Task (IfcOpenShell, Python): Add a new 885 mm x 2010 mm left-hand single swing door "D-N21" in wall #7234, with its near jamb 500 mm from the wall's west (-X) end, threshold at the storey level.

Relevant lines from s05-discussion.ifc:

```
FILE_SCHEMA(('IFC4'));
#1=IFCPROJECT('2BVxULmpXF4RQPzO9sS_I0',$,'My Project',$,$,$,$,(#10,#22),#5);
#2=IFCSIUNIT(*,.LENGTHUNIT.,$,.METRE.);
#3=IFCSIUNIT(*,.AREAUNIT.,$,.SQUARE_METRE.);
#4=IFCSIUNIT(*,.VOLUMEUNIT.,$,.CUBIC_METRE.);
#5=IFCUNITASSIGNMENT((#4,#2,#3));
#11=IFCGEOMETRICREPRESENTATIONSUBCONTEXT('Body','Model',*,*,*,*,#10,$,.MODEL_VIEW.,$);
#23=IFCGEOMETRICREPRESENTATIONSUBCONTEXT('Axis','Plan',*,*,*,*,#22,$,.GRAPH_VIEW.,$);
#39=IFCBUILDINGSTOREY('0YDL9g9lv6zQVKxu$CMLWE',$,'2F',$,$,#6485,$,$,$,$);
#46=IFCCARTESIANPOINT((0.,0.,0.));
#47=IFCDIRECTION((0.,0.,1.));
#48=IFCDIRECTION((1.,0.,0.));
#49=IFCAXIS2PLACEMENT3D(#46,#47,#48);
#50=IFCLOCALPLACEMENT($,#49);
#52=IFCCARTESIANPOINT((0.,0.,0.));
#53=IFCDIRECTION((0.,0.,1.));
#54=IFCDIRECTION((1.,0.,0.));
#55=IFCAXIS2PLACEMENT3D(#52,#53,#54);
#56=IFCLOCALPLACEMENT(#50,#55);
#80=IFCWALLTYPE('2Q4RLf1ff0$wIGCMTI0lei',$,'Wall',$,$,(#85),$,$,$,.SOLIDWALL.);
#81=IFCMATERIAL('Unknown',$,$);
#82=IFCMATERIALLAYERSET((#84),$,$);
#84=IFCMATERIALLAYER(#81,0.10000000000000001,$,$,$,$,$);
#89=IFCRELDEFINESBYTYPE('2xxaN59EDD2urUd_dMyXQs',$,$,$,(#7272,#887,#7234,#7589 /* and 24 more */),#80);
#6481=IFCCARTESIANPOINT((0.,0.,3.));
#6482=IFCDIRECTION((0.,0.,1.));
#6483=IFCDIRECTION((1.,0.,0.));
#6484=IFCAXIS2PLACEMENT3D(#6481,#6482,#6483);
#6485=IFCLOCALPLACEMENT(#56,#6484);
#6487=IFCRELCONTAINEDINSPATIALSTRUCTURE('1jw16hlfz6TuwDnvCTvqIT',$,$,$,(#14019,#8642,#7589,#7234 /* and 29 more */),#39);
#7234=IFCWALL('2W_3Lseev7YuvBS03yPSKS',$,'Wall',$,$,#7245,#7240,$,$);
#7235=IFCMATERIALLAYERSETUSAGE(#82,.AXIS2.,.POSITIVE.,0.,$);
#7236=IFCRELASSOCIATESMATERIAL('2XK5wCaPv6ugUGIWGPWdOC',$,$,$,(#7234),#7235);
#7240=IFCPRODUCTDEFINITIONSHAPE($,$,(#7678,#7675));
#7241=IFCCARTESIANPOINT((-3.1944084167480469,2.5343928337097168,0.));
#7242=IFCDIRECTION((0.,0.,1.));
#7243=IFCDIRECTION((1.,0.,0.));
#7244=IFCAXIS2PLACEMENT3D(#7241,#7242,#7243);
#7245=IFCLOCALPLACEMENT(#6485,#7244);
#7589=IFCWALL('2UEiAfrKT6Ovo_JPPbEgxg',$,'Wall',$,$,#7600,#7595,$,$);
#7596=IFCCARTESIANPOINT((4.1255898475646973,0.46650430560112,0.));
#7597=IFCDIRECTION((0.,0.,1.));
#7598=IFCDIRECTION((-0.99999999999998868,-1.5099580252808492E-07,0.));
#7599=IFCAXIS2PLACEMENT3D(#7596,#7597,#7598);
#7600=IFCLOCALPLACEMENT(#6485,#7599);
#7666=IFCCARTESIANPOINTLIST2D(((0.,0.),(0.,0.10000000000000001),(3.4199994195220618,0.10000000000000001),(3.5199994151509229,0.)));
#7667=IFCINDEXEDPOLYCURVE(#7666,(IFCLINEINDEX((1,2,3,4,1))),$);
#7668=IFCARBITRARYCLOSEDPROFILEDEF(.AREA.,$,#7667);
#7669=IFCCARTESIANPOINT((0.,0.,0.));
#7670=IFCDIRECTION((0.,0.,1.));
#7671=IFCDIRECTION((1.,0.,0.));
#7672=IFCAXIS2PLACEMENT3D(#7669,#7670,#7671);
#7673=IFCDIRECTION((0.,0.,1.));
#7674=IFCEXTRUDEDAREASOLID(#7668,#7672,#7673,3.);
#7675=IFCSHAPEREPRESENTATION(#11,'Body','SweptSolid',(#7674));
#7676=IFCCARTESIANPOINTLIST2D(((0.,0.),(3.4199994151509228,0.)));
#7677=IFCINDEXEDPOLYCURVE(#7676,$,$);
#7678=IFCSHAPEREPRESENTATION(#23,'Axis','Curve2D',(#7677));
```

```python
import numpy as np
import ifcopenshell
import ifcopenshell.api.feature
import ifcopenshell.api.geometry
import ifcopenshell.api.root
import ifcopenshell.api.spatial
import ifcopenshell.geom
import ifcopenshell.util.element
import ifcopenshell.util.placement
import ifcopenshell.util.representation
import ifcopenshell.util.shape
import ifcopenshell.util.unit

model = ifcopenshell.open("s05-discussion.ifc")
unit_scale = ifcopenshell.util.unit.calculate_unit_scale(model)
settings = ifcopenshell.geom.settings()


def volume(element):
    """Net volume in cubic metres, openings subtracted."""
    shape = ifcopenshell.geom.create_shape(settings, element)
    return ifcopenshell.util.shape.get_volume(shape.geometry)


wall = model.by_guid("2W_3Lseev7YuvBS03yPSKS")
storey = ifcopenshell.util.element.get_container(wall, ifc_class="IfcBuildingStorey")
context = ifcopenshell.util.representation.get_context(model, "Model", "Body", "MODEL_VIEW")
before = volume(wall)

width, height, from_end, sill = 0.885, 2.01, 0.5, 0.0  # metres

# The wall runs along its own X axis, and the end named is its -X end.
wall_shape = ifcopenshell.geom.create_shape(settings, wall)
x, y, z = ifcopenshell.util.shape.get_vertices(wall_shape.geometry).T
start = x.min() + from_end
face, thickness = float(y.min()), float(y.max() - y.min())
wall_matrix = ifcopenshell.util.placement.get_local_placement(wall.ObjectPlacement)
level = ifcopenshell.util.placement.get_local_placement(storey.ObjectPlacement)[2, 3]


def in_wall(x, y):
    """Placement at x, y metres in the wall's axes, at sill height."""
    matrix = wall_matrix.copy()
    matrix[:, 3] = wall_matrix @ np.array([x / unit_scale, y / unit_scale, 0.0, 1.0])
    matrix[2, 3] = level + sill / unit_scale
    return matrix


# Opening: a box that overshoots both wall faces by 50 mm.
opening = ifcopenshell.api.root.create_entity(model, ifc_class="IfcOpeningElement", predefined_type="OPENING")
box = ifcopenshell.api.geometry.add_wall_representation(
    model, context=context, length=width, height=height, thickness=thickness + 0.1
)
ifcopenshell.api.geometry.assign_representation(model, product=opening, representation=box)
ifcopenshell.api.geometry.edit_object_placement(model, product=opening, matrix=in_wall(start, face - 0.05), is_si=False)
ifcopenshell.api.feature.add_feature(model, feature=opening, element=wall)

door = ifcopenshell.api.root.create_entity(model, ifc_class="IfcDoor", name="D-N21", predefined_type="DOOR")
door.OverallWidth, door.OverallHeight = width / unit_scale, height / unit_scale
door.OperationType = "SINGLE_SWING_LEFT"
body = ifcopenshell.api.geometry.add_door_representation(
    model,
    context=context,
    overall_width=door.OverallWidth,
    overall_height=door.OverallHeight,
    operation_type="SINGLE_SWING_LEFT",
    lining_properties={"LiningDepth": thickness / unit_scale, "ThresholdDepth": thickness / unit_scale},
)
ifcopenshell.api.geometry.assign_representation(model, product=door, representation=body)
ifcopenshell.api.spatial.assign_container(model, products=[door], relating_structure=storey)
ifcopenshell.api.feature.add_filling(model, opening=opening, element=door)

# The lining spans the wall, so the door starts at the wall face.
ifcopenshell.api.geometry.edit_object_placement(model, product=door, matrix=in_wall(start, face), is_si=False)

after = volume(wall)

print(f"wall volume {before:.3f} -> {after:.3f} m3")

model.write("s05-discussion_v2.ifc")
```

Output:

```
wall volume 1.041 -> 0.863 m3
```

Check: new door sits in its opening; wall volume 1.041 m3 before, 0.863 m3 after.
